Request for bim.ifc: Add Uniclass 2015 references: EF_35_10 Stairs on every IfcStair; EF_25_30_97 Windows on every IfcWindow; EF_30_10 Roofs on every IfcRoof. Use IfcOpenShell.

First a look at what the model holds.

```python
import ifcopenshell

model = ifcopenshell.open("bim.ifc")
print(model.schema)
print("classifications:", [c.Name for c in model.by_type("IfcClassification")])
for ifc_class in ("IfcDoor", "IfcRoof", "IfcStair", "IfcWall", "IfcWindow"):
    print(ifc_class, len(model.by_type(ifc_class)))
```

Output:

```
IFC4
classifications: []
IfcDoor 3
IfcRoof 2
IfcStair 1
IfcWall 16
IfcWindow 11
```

```python
import ifcopenshell
import ifcopenshell.api.classification

model = ifcopenshell.open("bim.ifc")

system = ifcopenshell.api.classification.add_classification(model, classification="Uniclass 2015")

codes = {
    "IfcStair": ("EF_35_10", "Stairs"),
    "IfcWindow": ("EF_25_30_97", "Windows"),
    "IfcRoof": ("EF_30_10", "Roofs"),
}
for ifc_class, (code, name) in codes.items():
    products = model.by_type(ifc_class)
    ifcopenshell.api.classification.add_reference(
        model, products=products, classification=system, identification=code, name=name
    )
    print(code, len(products))

model.write("bim_updated.ifc")
```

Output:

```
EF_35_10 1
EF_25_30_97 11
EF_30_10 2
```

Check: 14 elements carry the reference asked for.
